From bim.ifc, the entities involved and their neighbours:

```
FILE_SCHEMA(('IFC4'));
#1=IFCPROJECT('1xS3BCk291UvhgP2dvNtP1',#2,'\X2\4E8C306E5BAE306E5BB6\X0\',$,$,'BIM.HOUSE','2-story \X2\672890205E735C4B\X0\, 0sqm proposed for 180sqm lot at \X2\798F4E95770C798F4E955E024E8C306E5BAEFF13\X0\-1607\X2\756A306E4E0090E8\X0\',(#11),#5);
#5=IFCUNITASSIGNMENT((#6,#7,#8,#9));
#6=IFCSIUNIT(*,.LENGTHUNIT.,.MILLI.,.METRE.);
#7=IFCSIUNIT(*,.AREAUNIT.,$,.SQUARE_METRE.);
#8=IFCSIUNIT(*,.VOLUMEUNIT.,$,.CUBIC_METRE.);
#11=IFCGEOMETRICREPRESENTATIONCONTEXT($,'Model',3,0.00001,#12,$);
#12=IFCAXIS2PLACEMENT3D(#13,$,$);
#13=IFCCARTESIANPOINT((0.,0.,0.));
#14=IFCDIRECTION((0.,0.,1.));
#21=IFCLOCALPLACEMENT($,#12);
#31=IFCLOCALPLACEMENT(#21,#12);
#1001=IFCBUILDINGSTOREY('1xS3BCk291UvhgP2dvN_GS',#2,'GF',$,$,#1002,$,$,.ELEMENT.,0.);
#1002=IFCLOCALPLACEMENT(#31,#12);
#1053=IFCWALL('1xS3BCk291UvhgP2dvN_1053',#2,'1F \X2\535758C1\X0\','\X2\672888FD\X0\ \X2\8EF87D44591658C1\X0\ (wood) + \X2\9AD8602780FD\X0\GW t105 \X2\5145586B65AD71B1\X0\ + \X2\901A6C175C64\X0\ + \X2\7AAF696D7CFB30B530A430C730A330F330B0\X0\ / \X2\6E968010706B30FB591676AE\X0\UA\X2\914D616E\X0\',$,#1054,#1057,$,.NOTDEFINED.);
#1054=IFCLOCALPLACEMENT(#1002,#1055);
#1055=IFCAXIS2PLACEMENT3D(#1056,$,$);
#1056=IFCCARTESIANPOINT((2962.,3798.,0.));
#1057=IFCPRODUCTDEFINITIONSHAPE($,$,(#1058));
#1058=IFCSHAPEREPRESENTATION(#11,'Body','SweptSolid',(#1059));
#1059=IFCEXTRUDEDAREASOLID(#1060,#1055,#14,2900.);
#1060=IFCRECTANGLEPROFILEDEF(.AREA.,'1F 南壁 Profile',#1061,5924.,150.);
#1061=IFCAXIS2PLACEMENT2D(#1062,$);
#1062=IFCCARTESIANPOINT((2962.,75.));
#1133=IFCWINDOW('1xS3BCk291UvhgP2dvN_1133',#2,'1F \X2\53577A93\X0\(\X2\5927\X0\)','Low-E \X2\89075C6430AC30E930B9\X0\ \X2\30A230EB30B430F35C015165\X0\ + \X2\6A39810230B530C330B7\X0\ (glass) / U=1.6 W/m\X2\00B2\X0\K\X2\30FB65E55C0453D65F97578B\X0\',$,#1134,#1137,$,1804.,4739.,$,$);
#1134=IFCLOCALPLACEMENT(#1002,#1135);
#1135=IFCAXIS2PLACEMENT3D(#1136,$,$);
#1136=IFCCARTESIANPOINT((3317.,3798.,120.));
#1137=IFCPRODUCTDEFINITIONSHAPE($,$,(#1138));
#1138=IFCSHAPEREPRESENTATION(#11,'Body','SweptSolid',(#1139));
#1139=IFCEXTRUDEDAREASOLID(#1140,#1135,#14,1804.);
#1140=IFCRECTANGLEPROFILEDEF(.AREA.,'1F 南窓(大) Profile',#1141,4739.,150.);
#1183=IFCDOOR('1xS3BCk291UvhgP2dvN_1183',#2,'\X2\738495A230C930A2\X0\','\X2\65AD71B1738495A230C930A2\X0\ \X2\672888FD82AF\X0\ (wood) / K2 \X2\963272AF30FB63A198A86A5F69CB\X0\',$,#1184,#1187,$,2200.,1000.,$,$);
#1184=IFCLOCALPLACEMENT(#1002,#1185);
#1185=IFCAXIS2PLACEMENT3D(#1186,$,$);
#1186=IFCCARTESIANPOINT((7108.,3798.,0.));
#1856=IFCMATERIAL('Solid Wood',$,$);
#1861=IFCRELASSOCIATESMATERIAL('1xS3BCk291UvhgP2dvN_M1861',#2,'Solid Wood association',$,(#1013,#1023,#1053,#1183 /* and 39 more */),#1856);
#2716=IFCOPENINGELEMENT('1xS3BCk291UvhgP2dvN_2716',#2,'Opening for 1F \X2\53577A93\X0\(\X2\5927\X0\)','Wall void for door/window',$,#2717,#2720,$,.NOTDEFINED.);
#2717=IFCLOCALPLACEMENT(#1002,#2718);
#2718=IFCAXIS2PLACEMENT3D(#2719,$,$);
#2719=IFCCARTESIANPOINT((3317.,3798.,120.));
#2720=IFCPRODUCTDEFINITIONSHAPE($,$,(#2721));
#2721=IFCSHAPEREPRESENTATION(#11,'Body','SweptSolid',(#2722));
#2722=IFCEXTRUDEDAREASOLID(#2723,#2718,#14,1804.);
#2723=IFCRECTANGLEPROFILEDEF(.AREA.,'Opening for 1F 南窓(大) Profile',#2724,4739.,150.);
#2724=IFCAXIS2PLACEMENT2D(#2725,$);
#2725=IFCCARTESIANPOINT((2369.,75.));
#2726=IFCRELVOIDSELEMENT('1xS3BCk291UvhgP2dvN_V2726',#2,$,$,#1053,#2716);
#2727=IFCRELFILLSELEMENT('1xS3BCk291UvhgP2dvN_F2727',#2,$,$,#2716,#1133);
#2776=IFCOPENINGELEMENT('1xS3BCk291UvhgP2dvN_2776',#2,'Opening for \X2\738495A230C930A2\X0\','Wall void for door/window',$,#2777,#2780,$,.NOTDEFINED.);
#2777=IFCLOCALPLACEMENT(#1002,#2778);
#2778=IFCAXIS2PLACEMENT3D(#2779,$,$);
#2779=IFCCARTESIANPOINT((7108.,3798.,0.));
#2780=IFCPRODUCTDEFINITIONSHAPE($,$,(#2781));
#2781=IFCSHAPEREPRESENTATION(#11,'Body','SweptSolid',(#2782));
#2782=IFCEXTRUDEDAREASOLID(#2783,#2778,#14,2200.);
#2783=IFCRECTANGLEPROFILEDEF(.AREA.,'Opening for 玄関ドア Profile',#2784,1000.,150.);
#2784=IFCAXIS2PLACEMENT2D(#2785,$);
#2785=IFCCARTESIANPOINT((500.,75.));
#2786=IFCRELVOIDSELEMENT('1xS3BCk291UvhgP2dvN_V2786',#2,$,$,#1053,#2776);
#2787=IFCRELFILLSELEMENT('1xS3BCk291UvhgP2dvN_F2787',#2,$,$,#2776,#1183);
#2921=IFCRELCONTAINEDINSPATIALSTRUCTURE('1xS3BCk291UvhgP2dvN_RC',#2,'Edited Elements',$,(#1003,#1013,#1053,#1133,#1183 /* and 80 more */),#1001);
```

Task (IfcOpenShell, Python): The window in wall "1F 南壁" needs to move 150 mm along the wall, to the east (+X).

```python
import ifcopenshell
import ifcopenshell.api.geometry
import ifcopenshell.util.placement
import ifcopenshell.util.unit

model = ifcopenshell.open("bim.ifc")
unit_scale = ifcopenshell.util.unit.calculate_unit_scale(model)

window = model.by_id(1133)
opening = window.FillsVoids[0].RelatingOpeningElement
wall = opening.VoidsElements[0].RelatingBuildingElement

wall_matrix = ifcopenshell.util.placement.get_local_placement(wall.ObjectPlacement)
shift = wall_matrix[:3, 0] * 0.15 / unit_scale
before = ifcopenshell.util.placement.get_local_placement(window.ObjectPlacement)[:3, 3].copy()

# The window is not placed relative to its opening, so move both.
for product in (opening, window):
    matrix = ifcopenshell.util.placement.get_local_placement(product.ObjectPlacement)
    matrix[:3, 3] += shift
    ifcopenshell.api.geometry.edit_object_placement(model, product=product, matrix=matrix, is_si=False)

after = ifcopenshell.util.placement.get_local_placement(window.ObjectPlacement)[:3, 3]
print("window moved by", (after - before).round(3) + 0.0)

model.write("bim_edited.ifc")
```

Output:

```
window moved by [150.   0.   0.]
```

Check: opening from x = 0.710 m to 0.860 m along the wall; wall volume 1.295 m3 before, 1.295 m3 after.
